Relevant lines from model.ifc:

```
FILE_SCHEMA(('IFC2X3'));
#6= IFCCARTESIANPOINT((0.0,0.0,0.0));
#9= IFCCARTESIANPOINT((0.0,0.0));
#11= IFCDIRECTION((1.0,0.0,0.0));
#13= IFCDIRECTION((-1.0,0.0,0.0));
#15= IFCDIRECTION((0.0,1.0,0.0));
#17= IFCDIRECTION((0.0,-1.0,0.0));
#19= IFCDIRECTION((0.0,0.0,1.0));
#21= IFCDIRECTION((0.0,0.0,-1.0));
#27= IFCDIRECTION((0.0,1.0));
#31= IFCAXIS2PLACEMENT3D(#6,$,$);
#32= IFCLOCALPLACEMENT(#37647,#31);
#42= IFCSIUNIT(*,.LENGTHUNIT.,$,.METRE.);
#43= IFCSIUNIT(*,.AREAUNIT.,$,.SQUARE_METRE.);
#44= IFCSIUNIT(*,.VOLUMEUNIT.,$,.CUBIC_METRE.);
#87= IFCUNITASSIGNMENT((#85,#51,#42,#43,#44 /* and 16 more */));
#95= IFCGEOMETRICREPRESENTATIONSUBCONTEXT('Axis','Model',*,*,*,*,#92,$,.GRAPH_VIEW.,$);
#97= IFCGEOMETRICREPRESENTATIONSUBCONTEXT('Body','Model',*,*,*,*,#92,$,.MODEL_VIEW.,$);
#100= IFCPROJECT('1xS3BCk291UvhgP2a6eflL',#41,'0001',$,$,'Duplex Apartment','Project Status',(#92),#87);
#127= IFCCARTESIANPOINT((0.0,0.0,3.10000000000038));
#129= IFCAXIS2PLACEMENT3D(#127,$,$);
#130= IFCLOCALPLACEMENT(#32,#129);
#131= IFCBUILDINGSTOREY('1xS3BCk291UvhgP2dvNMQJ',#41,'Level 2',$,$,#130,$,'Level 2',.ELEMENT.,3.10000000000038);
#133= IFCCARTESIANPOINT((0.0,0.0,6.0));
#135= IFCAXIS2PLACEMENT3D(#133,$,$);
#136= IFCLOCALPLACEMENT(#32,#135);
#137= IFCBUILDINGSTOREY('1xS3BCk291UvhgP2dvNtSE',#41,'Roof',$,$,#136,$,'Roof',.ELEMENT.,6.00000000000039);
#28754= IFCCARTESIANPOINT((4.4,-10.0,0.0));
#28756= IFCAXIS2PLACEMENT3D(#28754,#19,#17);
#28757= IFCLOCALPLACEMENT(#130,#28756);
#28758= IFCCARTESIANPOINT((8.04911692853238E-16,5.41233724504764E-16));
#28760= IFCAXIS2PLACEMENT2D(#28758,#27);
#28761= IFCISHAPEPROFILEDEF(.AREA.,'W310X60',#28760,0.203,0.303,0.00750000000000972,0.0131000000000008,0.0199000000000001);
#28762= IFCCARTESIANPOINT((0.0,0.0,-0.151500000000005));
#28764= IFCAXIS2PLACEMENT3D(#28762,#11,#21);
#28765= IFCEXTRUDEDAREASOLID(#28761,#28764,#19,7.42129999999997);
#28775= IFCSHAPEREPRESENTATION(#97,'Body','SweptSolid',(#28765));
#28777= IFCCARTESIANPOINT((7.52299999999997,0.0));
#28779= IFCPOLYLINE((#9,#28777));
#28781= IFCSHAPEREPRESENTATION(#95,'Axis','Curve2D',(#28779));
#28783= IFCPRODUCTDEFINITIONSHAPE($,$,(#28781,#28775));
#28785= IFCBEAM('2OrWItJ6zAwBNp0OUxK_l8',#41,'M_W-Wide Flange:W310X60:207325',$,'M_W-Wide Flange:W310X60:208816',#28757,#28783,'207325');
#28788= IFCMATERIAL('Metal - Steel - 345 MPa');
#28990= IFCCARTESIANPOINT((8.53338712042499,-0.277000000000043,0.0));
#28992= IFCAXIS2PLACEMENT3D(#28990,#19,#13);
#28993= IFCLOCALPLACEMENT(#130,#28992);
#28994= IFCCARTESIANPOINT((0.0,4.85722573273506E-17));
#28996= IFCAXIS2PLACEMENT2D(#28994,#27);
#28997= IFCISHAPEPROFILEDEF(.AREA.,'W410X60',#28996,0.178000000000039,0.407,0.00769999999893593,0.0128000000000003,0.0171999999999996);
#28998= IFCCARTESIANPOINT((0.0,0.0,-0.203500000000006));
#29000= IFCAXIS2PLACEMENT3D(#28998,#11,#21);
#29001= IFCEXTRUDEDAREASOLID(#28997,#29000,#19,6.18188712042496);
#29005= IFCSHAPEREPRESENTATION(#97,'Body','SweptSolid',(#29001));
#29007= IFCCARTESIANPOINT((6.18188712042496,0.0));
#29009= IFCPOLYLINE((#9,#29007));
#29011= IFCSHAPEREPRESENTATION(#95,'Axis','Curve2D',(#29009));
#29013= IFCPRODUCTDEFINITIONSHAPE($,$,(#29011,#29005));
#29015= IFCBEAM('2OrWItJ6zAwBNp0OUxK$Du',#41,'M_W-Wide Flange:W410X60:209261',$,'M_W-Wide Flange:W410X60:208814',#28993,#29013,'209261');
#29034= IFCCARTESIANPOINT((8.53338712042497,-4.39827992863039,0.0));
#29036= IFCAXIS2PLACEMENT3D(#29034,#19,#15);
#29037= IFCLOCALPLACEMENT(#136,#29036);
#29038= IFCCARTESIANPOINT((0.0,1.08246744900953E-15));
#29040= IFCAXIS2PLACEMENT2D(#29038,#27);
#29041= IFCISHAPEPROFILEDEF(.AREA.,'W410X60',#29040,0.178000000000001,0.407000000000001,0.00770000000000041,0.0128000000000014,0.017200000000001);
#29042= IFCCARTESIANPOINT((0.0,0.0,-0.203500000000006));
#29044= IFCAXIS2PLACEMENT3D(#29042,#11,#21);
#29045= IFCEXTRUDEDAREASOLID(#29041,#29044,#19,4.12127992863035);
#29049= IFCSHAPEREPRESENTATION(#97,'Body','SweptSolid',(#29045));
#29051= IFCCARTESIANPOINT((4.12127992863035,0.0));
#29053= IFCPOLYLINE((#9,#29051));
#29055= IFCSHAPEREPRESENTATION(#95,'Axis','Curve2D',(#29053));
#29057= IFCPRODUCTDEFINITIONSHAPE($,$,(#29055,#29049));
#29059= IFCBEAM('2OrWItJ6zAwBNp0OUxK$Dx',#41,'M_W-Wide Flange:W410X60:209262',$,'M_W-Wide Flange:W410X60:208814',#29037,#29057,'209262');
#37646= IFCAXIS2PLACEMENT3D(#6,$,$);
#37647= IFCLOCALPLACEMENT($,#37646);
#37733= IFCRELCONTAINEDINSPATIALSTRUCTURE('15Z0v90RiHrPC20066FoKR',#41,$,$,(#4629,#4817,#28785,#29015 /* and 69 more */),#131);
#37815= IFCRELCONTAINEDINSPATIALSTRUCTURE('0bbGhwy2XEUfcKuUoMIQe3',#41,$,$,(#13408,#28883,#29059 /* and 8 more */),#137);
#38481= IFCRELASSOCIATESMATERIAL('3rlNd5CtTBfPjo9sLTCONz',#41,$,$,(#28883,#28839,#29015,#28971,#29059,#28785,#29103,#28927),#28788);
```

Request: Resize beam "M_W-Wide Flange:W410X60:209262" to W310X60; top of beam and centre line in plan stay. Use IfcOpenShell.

```python
import ifcopenshell
import ifcopenshell.util.element
import ifcopenshell.util.representation

model = ifcopenshell.open("model.ifc")

member = model.by_id(29059)
source = next(p for p in model.by_type("IfcIShapeProfileDef") if p.ProfileName == "W310X60")

body = ifcopenshell.util.representation.get_representation(member, "Model", "Body")
solid = body.Items[0]
old_profile = solid.SweptArea

# Copy the section's sizes but keep this member's own profile position.
profile = ifcopenshell.util.element.copy(model, source)
# Profiles are centred, so shift by half the change in depth to hold the top.
shift = (old_profile.OverallDepth - profile.OverallDepth) / 2
x, y = old_profile.Position.Location.Coordinates
up = (-1.0, 0.0)  # upwards, in the solid's own plane
location = model.createIfcCartesianPoint((x + up[0] * shift, y + up[1] * shift))
profile.Position = model.createIfcAxis2Placement2D(location, old_profile.Position.RefDirection)
solid.SweptArea = profile
if not model.get_total_inverses(old_profile):
    ifcopenshell.util.element.remove_deep2(model, old_profile)
member.Name = member.Name.replace("W410X60", "W310X60")
member.ObjectType = member.ObjectType.replace("W410X60", "W310X60")

print(solid.SweptArea)

model.write("model_updated.ifc")
```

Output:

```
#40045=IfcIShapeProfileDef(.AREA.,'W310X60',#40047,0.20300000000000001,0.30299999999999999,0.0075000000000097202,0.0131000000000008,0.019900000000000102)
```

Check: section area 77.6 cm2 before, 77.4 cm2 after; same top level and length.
